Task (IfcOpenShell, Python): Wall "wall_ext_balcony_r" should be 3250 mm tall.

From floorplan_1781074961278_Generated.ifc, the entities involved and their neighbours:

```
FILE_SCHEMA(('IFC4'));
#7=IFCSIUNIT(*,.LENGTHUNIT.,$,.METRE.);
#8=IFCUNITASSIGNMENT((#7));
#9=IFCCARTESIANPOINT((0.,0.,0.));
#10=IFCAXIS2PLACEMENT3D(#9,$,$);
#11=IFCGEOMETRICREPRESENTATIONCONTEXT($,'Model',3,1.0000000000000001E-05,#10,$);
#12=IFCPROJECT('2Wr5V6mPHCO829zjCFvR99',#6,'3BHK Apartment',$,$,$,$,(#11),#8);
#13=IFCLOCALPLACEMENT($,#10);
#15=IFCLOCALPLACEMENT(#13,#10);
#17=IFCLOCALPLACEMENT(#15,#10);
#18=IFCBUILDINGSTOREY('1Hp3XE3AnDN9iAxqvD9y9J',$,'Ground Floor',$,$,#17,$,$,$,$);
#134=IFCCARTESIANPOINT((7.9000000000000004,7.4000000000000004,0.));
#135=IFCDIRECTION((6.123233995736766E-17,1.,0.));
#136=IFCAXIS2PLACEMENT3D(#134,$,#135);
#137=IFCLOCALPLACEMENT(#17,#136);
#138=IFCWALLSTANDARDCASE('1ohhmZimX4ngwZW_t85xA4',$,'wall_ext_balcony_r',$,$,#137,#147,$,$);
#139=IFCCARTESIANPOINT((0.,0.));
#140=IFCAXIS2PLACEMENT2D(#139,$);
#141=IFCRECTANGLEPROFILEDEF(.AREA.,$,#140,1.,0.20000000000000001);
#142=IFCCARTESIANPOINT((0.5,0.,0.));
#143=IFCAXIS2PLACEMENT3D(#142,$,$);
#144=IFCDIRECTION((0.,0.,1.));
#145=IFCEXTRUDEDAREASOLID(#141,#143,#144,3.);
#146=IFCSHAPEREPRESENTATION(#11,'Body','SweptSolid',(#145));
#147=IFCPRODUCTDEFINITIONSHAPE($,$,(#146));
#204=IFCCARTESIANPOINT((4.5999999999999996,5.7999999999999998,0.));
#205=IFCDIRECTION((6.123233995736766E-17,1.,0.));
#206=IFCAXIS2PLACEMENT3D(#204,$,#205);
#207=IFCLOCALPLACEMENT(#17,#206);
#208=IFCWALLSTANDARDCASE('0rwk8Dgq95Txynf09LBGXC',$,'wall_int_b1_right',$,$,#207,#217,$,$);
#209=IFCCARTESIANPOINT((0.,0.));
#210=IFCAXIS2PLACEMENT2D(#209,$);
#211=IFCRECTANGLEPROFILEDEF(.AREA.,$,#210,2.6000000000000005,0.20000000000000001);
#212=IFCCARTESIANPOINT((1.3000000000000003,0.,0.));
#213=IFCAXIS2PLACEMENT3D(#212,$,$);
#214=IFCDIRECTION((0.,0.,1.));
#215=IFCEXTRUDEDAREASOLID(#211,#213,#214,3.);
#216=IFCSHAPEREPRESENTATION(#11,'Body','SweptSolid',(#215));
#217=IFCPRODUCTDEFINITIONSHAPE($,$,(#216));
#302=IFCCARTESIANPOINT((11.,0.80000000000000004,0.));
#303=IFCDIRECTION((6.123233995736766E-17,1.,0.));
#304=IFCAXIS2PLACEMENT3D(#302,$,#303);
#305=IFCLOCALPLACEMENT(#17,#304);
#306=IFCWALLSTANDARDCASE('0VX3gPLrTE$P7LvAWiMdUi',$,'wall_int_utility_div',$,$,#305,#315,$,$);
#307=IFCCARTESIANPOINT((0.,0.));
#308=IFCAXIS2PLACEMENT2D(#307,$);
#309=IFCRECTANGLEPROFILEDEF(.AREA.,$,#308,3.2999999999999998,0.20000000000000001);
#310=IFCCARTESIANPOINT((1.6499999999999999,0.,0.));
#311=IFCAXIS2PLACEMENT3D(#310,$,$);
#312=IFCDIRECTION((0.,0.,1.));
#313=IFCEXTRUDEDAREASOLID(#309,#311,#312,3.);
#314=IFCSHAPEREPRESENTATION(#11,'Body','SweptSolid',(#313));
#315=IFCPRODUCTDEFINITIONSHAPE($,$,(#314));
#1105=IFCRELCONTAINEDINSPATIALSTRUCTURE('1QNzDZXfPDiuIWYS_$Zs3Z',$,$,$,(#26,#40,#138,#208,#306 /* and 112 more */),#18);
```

```python
import ifcopenshell
import ifcopenshell.geom
import ifcopenshell.util.shape
import ifcopenshell.util.unit

model = ifcopenshell.open("floorplan_1781074961278_Generated.ifc")
unit_scale = ifcopenshell.util.unit.calculate_unit_scale(model)
settings = ifcopenshell.geom.settings()


def volume(element):
    """Net volume in cubic metres, openings subtracted."""
    shape = ifcopenshell.geom.create_shape(settings, element)
    return ifcopenshell.util.shape.get_volume(shape.geometry)


wall = model.by_guid("1ohhmZimX4ngwZW_t85xA4")
before = volume(wall)

body = next(r for r in wall.Representation.Representations if r.RepresentationIdentifier == "Body")
solid = body.Items[0]
old_height = solid.Depth
solid.Depth = 3.25 / unit_scale
after = volume(wall)

print(f"height {old_height:g} -> {solid.Depth:g}, volume {before:.3f} -> {after:.3f} m3")

model.write("floorplan_1781074961278_Generated_edited.ifc")
```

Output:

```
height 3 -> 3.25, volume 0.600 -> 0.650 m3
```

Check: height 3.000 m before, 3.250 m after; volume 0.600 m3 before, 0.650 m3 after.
